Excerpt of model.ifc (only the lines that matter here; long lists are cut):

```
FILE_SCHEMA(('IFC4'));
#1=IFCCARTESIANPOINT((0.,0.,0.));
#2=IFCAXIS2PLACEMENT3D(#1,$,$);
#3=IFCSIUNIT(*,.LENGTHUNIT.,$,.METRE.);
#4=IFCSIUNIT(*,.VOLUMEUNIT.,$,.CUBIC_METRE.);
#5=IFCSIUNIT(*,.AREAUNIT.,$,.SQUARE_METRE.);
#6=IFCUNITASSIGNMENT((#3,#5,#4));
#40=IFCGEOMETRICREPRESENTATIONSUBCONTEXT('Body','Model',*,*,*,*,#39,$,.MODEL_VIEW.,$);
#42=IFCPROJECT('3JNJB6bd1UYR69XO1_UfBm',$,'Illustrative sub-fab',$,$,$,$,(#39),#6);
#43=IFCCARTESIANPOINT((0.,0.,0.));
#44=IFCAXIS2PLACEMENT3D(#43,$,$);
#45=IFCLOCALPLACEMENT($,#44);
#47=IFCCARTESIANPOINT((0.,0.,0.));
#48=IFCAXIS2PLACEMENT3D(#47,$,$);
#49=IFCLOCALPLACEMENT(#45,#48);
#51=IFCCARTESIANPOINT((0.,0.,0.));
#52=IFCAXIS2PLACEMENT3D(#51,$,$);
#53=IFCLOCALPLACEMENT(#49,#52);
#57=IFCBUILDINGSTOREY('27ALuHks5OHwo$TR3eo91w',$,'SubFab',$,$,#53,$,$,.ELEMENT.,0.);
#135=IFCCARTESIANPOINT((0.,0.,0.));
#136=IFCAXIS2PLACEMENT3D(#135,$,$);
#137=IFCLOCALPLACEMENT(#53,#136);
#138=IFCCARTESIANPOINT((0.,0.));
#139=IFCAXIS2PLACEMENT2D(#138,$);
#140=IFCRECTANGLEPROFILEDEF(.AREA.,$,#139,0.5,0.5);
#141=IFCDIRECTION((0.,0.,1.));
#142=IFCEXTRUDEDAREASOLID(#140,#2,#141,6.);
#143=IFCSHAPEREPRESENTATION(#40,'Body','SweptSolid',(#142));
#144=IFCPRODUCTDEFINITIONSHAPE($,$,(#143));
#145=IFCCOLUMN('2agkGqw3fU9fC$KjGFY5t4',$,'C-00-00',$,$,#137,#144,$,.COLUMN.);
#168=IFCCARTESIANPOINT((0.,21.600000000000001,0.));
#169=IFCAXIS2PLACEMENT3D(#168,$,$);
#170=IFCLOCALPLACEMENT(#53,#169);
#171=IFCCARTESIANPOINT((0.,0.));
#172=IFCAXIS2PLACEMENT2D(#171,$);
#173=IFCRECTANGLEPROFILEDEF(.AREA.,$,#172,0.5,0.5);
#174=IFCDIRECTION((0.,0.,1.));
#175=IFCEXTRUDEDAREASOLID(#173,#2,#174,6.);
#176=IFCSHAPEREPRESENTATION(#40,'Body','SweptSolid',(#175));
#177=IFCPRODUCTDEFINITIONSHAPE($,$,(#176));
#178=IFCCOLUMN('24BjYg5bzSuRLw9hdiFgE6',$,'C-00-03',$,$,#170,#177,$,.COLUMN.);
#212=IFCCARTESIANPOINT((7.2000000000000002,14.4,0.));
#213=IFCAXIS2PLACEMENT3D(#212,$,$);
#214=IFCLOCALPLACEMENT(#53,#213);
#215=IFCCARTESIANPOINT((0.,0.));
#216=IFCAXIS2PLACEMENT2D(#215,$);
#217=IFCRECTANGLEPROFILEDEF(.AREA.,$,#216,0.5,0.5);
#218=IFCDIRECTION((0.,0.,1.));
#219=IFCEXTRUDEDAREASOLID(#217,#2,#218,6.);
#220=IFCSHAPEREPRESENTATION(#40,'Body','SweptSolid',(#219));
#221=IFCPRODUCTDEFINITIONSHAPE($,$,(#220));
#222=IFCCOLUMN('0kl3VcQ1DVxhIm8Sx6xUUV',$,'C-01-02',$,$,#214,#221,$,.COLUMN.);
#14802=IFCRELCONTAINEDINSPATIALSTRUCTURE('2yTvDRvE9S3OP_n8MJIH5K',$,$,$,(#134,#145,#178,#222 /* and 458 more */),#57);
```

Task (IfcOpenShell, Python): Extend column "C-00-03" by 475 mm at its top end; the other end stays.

```python
import ifcopenshell
import ifcopenshell.util.representation
import ifcopenshell.util.unit

model = ifcopenshell.open("model.ifc")
unit_scale = ifcopenshell.util.unit.calculate_unit_scale(model)

member = model.by_guid("24BjYg5bzSuRLw9hdiFgE6")
change = 0.475 / unit_scale

# The extrusion runs towards the end named, so only its depth changes.
body = ifcopenshell.util.representation.get_representation(member, "Model", "Body")
solid = body.Items[0]
old_length = solid.Depth
solid.Depth += change

print(f"length {old_length:g} -> {solid.Depth:g}")

model.write("model_updated.ifc")
```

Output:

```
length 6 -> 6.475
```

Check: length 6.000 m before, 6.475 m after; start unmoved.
